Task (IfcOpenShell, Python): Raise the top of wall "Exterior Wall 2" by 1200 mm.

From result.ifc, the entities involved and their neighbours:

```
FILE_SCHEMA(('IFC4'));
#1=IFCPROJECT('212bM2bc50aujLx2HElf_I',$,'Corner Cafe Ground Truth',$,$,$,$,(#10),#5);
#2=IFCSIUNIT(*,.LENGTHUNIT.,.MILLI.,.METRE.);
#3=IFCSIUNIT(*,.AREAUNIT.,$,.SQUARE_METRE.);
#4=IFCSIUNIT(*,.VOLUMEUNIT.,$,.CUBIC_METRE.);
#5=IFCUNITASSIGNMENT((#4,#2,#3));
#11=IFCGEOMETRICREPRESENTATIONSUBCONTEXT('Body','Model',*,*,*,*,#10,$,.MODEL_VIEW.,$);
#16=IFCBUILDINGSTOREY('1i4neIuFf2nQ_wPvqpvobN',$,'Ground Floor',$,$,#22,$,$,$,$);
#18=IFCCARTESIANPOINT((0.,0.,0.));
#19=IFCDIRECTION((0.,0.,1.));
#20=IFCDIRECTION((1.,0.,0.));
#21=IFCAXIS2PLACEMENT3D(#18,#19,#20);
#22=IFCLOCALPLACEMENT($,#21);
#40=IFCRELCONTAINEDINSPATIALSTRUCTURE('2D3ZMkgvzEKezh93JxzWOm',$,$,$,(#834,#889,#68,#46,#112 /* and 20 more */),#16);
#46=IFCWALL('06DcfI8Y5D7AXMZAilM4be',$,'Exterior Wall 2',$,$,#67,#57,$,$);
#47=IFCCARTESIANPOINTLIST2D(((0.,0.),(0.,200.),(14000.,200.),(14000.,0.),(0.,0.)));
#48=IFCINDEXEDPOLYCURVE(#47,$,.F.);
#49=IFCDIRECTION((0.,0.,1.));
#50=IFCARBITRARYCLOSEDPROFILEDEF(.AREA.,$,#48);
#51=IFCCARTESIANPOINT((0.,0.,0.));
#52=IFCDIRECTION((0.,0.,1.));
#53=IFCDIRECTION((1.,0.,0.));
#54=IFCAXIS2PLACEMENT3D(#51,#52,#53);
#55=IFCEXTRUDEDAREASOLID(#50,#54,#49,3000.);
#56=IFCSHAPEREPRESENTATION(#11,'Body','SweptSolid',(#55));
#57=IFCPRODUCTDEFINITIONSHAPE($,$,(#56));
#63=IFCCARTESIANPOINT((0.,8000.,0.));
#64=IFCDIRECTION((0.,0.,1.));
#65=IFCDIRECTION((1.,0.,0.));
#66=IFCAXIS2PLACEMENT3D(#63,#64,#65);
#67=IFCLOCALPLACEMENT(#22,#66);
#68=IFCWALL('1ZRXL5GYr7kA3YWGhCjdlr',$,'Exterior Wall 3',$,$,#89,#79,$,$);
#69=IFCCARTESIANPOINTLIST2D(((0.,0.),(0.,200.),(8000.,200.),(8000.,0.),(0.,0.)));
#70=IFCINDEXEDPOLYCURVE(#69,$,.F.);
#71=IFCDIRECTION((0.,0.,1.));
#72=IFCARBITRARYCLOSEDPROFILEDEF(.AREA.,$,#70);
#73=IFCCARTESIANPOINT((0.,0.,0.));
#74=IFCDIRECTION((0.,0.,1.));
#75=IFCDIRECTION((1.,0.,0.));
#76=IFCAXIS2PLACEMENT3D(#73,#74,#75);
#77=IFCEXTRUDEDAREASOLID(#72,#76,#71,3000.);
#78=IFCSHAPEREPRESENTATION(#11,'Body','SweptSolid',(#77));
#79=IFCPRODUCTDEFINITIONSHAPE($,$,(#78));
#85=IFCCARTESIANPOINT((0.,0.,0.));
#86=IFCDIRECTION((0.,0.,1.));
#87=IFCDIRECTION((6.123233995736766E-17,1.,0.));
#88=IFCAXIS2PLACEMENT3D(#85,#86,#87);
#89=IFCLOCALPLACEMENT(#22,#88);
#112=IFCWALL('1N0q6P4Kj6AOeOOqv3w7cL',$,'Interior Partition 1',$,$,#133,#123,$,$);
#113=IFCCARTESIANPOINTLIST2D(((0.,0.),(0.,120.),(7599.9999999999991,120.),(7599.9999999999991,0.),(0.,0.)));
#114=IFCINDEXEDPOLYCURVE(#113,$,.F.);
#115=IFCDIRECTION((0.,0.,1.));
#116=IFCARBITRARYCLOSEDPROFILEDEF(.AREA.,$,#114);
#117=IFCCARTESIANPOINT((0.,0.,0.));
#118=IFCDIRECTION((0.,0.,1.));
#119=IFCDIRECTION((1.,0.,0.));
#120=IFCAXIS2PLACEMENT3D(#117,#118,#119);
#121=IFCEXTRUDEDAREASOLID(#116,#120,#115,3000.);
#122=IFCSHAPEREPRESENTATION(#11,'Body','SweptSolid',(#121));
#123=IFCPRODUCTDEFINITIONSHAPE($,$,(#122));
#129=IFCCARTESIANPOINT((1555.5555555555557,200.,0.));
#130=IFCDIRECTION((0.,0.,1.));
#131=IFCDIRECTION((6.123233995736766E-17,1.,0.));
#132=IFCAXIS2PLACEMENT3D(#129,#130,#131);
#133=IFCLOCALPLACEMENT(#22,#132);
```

```python
import ifcopenshell
import ifcopenshell.geom
import ifcopenshell.util.representation
import ifcopenshell.util.shape
import ifcopenshell.util.unit

model = ifcopenshell.open("result.ifc")
unit_scale = ifcopenshell.util.unit.calculate_unit_scale(model)
settings = ifcopenshell.geom.settings()


def volume(element):
    """Net volume in cubic metres, openings subtracted."""
    shape = ifcopenshell.geom.create_shape(settings, element)
    return ifcopenshell.util.shape.get_volume(shape.geometry)


wall = model.by_guid("06DcfI8Y5D7AXMZAilM4be")
before = volume(wall)

body = ifcopenshell.util.representation.get_representation(wall, "Model", "Body")
solid = body.Items[0]
old_height = solid.Depth
solid.Depth += 1.2 / unit_scale
after = volume(wall)

print(f"height {old_height:g} -> {solid.Depth:g}, volume {before:.3f} -> {after:.3f} m3")

model.write("result_v2.ifc")
```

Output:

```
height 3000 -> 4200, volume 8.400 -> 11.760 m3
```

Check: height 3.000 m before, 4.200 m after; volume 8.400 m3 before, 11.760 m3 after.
